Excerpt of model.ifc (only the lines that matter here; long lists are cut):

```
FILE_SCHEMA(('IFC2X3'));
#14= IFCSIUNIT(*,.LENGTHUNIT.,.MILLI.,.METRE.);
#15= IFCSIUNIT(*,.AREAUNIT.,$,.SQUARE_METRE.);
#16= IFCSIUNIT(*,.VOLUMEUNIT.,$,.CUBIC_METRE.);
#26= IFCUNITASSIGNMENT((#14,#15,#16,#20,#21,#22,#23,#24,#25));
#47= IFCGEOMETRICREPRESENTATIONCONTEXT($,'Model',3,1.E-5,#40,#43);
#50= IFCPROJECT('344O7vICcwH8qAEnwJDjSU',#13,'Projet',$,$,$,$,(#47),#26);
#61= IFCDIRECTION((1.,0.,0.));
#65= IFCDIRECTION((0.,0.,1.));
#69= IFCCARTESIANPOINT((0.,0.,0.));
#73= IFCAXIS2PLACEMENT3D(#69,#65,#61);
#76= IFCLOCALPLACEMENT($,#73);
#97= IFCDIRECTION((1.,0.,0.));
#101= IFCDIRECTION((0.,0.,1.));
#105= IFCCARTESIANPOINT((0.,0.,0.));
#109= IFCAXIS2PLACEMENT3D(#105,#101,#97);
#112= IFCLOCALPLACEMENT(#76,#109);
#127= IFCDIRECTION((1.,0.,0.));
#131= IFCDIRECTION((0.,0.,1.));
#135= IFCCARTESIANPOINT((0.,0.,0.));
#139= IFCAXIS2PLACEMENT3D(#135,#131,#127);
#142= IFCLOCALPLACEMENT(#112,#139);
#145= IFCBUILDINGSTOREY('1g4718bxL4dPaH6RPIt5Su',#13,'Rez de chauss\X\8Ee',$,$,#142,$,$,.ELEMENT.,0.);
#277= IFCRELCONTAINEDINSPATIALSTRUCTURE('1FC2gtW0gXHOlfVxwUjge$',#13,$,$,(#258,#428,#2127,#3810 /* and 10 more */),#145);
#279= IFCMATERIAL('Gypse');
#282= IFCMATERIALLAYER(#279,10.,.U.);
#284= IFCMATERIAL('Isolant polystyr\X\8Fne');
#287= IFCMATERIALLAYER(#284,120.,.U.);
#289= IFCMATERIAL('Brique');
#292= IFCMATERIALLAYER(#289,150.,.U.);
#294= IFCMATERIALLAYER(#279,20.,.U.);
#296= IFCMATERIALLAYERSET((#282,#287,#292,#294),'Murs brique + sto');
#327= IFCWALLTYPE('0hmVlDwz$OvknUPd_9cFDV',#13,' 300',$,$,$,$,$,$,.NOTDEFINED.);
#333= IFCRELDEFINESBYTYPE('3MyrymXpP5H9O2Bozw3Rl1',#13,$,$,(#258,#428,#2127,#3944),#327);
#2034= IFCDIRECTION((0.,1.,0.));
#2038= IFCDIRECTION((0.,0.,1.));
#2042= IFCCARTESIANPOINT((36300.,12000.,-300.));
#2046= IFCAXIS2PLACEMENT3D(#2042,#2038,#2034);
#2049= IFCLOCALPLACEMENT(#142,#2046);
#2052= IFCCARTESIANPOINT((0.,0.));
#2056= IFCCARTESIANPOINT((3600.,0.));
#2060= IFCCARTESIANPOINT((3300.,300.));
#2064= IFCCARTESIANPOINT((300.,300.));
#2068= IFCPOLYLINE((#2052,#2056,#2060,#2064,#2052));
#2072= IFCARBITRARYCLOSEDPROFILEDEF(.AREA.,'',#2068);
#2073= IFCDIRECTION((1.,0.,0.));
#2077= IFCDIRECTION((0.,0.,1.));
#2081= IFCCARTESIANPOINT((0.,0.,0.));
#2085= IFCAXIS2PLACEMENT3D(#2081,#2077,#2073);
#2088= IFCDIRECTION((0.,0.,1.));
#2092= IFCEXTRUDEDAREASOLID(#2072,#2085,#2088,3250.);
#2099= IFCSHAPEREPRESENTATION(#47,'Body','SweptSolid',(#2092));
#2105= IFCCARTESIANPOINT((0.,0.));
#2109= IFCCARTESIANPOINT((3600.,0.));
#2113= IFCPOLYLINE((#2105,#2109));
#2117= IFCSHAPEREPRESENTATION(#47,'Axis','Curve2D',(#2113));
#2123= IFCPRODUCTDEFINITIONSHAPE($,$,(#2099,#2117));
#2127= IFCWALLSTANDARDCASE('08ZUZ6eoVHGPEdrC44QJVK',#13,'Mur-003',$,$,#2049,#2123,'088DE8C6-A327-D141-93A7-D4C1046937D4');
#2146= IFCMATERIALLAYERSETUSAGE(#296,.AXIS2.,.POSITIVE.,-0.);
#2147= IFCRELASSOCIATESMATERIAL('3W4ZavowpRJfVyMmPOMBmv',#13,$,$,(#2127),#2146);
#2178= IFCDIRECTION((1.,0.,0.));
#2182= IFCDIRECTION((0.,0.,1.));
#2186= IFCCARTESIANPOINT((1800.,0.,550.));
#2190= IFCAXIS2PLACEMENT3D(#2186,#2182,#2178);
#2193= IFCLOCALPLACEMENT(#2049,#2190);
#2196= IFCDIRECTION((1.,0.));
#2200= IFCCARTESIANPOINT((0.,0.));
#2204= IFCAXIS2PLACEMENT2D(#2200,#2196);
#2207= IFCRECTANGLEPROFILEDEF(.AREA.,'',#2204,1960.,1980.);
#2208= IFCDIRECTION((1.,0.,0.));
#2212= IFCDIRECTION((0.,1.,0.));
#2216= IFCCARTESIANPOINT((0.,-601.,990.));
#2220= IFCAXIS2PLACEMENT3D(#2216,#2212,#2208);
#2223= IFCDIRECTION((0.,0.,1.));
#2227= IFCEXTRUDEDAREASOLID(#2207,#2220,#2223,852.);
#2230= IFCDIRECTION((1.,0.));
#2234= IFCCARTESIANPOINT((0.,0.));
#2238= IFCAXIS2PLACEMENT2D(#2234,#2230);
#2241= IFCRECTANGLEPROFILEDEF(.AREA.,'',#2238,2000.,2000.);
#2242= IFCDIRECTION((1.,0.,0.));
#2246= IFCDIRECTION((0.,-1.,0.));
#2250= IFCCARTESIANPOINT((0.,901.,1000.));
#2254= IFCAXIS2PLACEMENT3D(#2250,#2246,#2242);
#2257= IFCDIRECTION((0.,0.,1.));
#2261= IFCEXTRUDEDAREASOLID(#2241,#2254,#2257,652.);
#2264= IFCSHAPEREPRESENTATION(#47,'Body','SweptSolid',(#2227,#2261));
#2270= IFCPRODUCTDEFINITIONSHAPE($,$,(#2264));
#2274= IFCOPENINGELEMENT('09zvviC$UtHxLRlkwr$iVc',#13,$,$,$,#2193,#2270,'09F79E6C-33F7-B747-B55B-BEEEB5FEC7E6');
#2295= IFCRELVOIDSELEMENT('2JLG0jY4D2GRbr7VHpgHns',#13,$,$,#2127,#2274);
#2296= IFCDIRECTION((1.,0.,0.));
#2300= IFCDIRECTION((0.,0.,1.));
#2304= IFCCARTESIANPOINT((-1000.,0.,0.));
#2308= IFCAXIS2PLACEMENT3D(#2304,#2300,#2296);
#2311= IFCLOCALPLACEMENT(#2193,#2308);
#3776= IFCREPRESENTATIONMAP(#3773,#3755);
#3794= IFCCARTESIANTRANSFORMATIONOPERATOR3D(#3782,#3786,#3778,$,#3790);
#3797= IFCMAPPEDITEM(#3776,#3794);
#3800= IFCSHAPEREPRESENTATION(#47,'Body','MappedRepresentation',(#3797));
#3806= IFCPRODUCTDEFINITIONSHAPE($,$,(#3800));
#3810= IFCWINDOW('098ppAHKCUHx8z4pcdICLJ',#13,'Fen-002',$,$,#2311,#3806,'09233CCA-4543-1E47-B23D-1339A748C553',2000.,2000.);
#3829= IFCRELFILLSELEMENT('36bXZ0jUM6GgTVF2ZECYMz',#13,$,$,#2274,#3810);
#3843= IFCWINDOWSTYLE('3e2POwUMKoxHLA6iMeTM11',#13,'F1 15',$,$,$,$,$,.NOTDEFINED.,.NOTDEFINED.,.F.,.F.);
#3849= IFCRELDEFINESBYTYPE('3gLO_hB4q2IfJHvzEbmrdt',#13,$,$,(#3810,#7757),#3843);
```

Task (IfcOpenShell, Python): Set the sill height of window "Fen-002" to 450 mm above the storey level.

```python
import numpy as np
import ifcopenshell
import ifcopenshell.api.geometry
import ifcopenshell.geom
import ifcopenshell.util.element
import ifcopenshell.util.placement
import ifcopenshell.util.shape
import ifcopenshell.util.unit

model = ifcopenshell.open("model.ifc")
unit_scale = ifcopenshell.util.unit.calculate_unit_scale(model)

window = model.by_guid("098ppAHKCUHx8z4pcdICLJ")
opening = window.FillsVoids[0].RelatingOpeningElement
storey = ifcopenshell.util.element.get_container(window, ifc_class="IfcBuildingStorey")
level = ifcopenshell.util.placement.get_local_placement(storey.ObjectPlacement)[2, 3]

# The opening's origin need not be at the sill, so measure its lowest point.
shape = ifcopenshell.geom.create_shape(ifcopenshell.geom.settings(), opening)
bottom = ifcopenshell.util.shape.get_shape_bottom_elevation(shape, shape.geometry) / unit_scale
dz = level + 450.0 - bottom

shift = np.array([0.0, 0.0, dz])
# The window is placed relative to its opening, so it follows when the opening moves.
matrix = ifcopenshell.util.placement.get_local_placement(opening.ObjectPlacement)
matrix[:3, 3] += shift
ifcopenshell.api.geometry.edit_object_placement(
    model, product=opening, matrix=matrix, is_si=False, should_transform_children=True
)

print(f"moved by {dz * unit_scale:+.3f} m")

model.write("model-out.ifc")
```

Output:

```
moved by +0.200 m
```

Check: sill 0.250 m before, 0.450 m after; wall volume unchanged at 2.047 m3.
